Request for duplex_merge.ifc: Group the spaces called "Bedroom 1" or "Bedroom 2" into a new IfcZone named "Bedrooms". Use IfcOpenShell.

First a look at what the model holds.

```python
import ifcopenshell

model = ifcopenshell.open("duplex_merge.ifc")
print(model.schema)
seen = {}
for space in model.by_type("IfcSpace"):
    seen[space.LongName] = seen.get(space.LongName, 0) + 1
for name, count in sorted(seen.items(), key=str):
    print(count, "x", name)
print("zones:", [z.Name for z in model.by_type("IfcZone")][:20])
```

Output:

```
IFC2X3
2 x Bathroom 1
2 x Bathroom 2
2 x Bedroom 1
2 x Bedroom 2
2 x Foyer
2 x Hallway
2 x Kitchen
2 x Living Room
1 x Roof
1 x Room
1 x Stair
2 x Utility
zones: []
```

```python
import ifcopenshell
import ifcopenshell.api.group
import ifcopenshell.api.root

model = ifcopenshell.open("duplex_merge.ifc")

names = {"Bedroom 1", "Bedroom 2"}
spaces = [s for s in model.by_type("IfcSpace") if s.LongName in names]

zone = ifcopenshell.api.root.create_entity(model, ifc_class="IfcZone", name="Bedrooms")
ifcopenshell.api.group.assign_group(model, products=spaces, group=zone)
print(len(spaces), "spaces in", zone.Name)

model.write("duplex_merge_updated.ifc")
```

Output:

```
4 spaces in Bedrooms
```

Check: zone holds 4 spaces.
